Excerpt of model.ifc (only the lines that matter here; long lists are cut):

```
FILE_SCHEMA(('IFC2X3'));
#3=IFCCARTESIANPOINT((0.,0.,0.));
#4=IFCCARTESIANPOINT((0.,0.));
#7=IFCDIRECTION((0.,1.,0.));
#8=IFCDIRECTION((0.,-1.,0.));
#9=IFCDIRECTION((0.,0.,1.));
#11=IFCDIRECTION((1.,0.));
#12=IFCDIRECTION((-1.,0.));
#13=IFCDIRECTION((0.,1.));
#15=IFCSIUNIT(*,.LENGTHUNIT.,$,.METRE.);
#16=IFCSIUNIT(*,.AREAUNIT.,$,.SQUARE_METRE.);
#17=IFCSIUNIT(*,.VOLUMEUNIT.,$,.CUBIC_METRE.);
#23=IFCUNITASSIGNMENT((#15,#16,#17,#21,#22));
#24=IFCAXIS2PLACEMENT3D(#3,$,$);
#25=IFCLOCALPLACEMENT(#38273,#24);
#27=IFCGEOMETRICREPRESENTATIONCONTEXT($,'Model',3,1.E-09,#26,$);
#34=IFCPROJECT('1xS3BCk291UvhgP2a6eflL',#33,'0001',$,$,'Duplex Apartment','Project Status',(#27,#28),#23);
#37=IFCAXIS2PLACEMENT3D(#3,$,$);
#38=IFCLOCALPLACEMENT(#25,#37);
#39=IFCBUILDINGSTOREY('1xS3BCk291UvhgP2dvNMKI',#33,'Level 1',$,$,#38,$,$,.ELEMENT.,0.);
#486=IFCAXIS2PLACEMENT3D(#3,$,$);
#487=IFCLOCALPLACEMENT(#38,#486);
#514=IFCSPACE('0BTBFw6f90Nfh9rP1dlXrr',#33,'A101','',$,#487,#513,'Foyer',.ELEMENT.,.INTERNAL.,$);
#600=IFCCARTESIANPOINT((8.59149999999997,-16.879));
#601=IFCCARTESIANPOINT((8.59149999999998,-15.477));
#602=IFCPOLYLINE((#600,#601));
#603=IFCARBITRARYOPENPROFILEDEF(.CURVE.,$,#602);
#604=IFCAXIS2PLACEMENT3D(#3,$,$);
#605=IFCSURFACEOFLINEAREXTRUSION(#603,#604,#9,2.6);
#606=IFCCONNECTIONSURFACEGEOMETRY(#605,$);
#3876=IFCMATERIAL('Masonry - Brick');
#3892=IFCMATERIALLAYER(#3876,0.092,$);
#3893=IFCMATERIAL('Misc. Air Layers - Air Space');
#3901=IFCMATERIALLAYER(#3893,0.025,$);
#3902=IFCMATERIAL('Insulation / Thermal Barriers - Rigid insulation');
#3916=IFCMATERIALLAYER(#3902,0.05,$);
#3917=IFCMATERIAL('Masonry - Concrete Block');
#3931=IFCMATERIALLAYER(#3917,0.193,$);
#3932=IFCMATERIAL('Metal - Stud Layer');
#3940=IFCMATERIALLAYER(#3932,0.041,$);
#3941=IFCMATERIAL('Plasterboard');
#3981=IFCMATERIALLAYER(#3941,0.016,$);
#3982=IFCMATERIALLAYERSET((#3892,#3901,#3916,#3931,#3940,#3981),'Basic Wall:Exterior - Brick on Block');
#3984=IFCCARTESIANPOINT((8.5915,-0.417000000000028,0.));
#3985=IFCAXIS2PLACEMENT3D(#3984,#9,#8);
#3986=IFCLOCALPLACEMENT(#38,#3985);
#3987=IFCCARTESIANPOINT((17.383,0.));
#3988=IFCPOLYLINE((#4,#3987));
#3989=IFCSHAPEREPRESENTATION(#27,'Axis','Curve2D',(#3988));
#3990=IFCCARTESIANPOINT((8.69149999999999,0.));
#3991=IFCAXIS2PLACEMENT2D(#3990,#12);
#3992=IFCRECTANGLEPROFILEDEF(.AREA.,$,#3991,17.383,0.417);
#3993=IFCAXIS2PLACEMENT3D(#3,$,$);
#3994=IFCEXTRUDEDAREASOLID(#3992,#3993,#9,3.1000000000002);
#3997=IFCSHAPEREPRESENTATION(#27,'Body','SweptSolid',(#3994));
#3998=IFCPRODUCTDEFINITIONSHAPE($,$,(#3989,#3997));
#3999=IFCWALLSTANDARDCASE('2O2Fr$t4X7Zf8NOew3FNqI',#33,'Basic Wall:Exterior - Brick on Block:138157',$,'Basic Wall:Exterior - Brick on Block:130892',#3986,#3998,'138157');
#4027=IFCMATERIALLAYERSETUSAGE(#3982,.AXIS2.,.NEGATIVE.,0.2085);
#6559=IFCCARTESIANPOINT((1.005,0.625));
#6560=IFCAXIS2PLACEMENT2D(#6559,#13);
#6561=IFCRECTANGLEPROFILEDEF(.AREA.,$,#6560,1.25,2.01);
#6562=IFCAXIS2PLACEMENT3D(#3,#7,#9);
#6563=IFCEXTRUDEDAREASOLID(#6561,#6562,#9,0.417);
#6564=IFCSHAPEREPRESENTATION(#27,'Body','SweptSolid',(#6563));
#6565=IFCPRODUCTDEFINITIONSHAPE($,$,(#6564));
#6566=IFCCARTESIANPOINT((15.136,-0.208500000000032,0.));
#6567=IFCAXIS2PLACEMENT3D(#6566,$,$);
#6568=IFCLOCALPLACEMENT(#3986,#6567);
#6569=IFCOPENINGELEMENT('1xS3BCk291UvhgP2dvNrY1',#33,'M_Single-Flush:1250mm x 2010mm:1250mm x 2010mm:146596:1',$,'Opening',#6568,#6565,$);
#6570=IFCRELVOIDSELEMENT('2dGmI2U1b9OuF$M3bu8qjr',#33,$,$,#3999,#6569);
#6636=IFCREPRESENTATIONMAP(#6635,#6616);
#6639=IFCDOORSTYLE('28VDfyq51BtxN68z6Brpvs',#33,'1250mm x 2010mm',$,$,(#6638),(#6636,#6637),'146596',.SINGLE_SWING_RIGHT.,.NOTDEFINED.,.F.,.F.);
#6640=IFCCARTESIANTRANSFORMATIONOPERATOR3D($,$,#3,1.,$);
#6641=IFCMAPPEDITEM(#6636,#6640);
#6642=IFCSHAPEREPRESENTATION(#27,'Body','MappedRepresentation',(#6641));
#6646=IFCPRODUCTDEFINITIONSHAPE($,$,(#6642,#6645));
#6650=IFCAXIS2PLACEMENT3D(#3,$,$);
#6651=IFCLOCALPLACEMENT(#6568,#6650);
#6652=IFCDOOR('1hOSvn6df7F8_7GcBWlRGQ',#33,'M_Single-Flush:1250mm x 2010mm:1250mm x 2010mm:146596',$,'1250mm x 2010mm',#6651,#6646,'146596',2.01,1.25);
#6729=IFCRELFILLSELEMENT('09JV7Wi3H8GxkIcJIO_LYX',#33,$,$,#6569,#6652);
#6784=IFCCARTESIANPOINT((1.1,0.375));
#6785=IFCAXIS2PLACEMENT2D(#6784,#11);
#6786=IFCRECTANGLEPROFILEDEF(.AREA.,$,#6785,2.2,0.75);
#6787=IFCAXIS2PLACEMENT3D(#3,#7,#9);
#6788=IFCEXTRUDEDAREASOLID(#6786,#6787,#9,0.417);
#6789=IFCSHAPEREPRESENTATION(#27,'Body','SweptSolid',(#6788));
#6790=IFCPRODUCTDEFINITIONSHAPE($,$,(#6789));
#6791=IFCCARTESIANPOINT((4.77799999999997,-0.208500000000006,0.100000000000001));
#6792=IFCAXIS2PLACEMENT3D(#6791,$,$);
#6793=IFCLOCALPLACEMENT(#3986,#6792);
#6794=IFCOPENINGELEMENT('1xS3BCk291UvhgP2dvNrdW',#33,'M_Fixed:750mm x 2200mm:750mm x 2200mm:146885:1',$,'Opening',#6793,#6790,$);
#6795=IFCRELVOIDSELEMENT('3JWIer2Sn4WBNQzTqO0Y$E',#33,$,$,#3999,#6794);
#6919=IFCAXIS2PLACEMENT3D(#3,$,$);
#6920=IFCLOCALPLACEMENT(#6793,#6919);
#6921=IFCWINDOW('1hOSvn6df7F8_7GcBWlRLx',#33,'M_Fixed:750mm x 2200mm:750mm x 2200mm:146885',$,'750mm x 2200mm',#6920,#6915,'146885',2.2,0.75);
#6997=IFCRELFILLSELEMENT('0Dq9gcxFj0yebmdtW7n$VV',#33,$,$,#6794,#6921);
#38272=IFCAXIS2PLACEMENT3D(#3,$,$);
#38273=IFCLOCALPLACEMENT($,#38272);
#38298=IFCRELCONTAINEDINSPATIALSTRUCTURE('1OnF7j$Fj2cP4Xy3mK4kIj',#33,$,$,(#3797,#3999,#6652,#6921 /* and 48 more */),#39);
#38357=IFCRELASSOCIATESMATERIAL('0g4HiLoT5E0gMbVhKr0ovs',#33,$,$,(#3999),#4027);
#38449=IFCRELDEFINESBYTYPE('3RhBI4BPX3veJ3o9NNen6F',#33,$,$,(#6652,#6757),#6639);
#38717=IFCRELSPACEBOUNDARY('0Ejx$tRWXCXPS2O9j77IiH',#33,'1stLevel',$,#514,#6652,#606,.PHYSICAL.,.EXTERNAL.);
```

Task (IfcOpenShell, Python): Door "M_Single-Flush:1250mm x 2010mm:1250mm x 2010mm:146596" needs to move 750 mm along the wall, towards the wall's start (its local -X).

```python
import numpy as np
import ifcopenshell
import ifcopenshell.api.geometry
import ifcopenshell.util.placement

model = ifcopenshell.open("model.ifc")

door = model.by_guid("1hOSvn6df7F8_7GcBWlRGQ")
opening = door.FillsVoids[0].RelatingOpeningElement
wall = opening.VoidsElements[0].RelatingBuildingElement

wall_matrix = ifcopenshell.util.placement.get_local_placement(wall.ObjectPlacement)
shift = wall_matrix[:3, 0] * -0.75
before = ifcopenshell.util.placement.get_local_placement(door.ObjectPlacement)[:3, 3].copy()

# The door is placed relative to its opening, so it follows when the opening moves.
matrix = ifcopenshell.util.placement.get_local_placement(opening.ObjectPlacement)
matrix[:3, 3] += shift
ifcopenshell.api.geometry.edit_object_placement(
    model, product=opening, matrix=matrix, is_si=False, should_transform_children=True
)

# Space boundary surfaces are stored in each space's coordinates; move them too.
for rel in door.ProvidesBoundaries:
    if not rel.ConnectionGeometry:
        continue
    surface = rel.ConnectionGeometry.SurfaceOnRelatingElement
    space_matrix = ifcopenshell.util.placement.get_local_placement(rel.RelatingSpace.ObjectPlacement)
    point = np.array(surface.Position.Location.Coordinates) + space_matrix[:3, :3].T @ shift
    surface.Position = model.createIfcAxis2Placement3D(
        model.createIfcCartesianPoint(point.tolist()), surface.Position.Axis, surface.Position.RefDirection
    )

after = ifcopenshell.util.placement.get_local_placement(door.ObjectPlacement)[:3, 3]
print("door moved by", (after - before).round(3) + 0.0)

model.write("model_rev.ifc")
```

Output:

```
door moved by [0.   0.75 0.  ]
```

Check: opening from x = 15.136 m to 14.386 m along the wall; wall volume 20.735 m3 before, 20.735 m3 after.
